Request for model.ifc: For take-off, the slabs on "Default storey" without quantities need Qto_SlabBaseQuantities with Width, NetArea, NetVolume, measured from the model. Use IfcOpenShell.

First a look at what the model holds.

```python
import ifcopenshell
import ifcopenshell.util.element
import ifcopenshell.util.unit

model = ifcopenshell.open("model.ifc")
print(model.schema)
for unit_type in ("LENGTHUNIT", "AREAUNIT", "VOLUMEUNIT"):
    print(unit_type, ifcopenshell.util.unit.calculate_unit_scale(model, unit_type))
storey = next(s for s in model.by_type("IfcBuildingStorey") if s.Name == "Default storey")
slabs = [e for e in ifcopenshell.util.element.get_decomposition(storey) if e.is_a("IfcSlab")]
for e in sorted(slabs, key=lambda e: e.id()):
    print(e.id(), e.is_a(), e.Name, list(ifcopenshell.util.element.get_psets(e, qtos_only=True)), sep=" | ")
```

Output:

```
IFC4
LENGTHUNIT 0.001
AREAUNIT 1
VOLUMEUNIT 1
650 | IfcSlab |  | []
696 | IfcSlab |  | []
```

```python
import ifcopenshell
import ifcopenshell.api.pset
import ifcopenshell.geom
import ifcopenshell.util.element
import ifcopenshell.util.shape
import ifcopenshell.util.unit

model = ifcopenshell.open("model.ifc")
unit_scale = ifcopenshell.util.unit.calculate_unit_scale(model)
area_scale = ifcopenshell.util.unit.calculate_unit_scale(model, "AREAUNIT")
volume_scale = ifcopenshell.util.unit.calculate_unit_scale(model, "VOLUMEUNIT")
settings = ifcopenshell.geom.settings()

storey = next(s for s in model.by_type("IfcBuildingStorey") if s.Name == "Default storey")
slabs = [e for e in ifcopenshell.util.element.get_decomposition(storey) if e.is_a("IfcSlab")]

for e in sorted(slabs, key=lambda e: e.id()):
    if ifcopenshell.util.element.get_psets(e, qtos_only=True, should_inherit=False):
        continue
    # Geometry comes back in metres, in the element's own axes.
    shape = ifcopenshell.geom.create_shape(settings, e)
    values = {
        "Width": ifcopenshell.util.shape.get_z(shape.geometry) / unit_scale,
        "NetArea": ifcopenshell.util.shape.get_footprint_area(shape.geometry) / area_scale,
        "NetVolume": ifcopenshell.util.shape.get_volume(shape.geometry) / volume_scale,
    }
    qto = ifcopenshell.api.pset.add_qto(model, product=e, name="Qto_SlabBaseQuantities")
    ifcopenshell.api.pset.edit_qto(model, qto=qto, properties=values)
    print(e.id(), {k: round(v, 3) for k, v in values.items()})

model.write("model-out.ifc")
```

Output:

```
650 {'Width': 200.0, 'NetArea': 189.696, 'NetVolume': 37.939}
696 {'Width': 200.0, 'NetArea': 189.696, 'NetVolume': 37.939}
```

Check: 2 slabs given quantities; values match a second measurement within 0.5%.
